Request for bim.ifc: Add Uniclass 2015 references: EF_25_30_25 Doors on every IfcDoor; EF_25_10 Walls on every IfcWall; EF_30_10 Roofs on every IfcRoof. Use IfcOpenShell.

First a look at what the model holds.

```python
import ifcopenshell

model = ifcopenshell.open("bim.ifc")
print(model.schema)
print("classifications:", [c.Name for c in model.by_type("IfcClassification")])
for ifc_class in ("IfcDoor", "IfcRoof", "IfcStair", "IfcWall", "IfcWindow"):
    print(ifc_class, len(model.by_type(ifc_class)))
```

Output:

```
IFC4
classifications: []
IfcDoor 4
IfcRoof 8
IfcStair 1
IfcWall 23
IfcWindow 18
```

```python
import ifcopenshell
import ifcopenshell.api.classification

model = ifcopenshell.open("bim.ifc")

system = ifcopenshell.api.classification.add_classification(model, classification="Uniclass 2015")

codes = {
    "IfcDoor": ("EF_25_30_25", "Doors"),
    "IfcWall": ("EF_25_10", "Walls"),
    "IfcRoof": ("EF_30_10", "Roofs"),
}
for ifc_class, (code, name) in codes.items():
    products = model.by_type(ifc_class)
    ifcopenshell.api.classification.add_reference(
        model, products=products, classification=system, identification=code, name=name
    )
    print(code, len(products))

model.write("bim_edited.ifc")
```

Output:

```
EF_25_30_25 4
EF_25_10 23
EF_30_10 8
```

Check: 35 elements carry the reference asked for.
